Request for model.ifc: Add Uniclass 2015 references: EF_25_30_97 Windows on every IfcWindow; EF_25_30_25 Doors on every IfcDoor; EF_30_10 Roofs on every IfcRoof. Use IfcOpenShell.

First a look at what the model holds.

```python
import ifcopenshell

model = ifcopenshell.open("model.ifc")
print(model.schema)
print("classifications:", [c.Name for c in model.by_type("IfcClassification")])
for ifc_class in ("IfcDoor", "IfcRoof", "IfcStair", "IfcWall", "IfcWindow"):
    print(ifc_class, len(model.by_type(ifc_class)))
```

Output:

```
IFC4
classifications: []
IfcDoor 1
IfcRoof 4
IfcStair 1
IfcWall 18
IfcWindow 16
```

```python
import ifcopenshell
import ifcopenshell.api.classification

model = ifcopenshell.open("model.ifc")

system = ifcopenshell.api.classification.add_classification(model, classification="Uniclass 2015")

codes = {
    "IfcWindow": ("EF_25_30_97", "Windows"),
    "IfcDoor": ("EF_25_30_25", "Doors"),
    "IfcRoof": ("EF_30_10", "Roofs"),
}
for ifc_class, (code, name) in codes.items():
    products = model.by_type(ifc_class)
    ifcopenshell.api.classification.add_reference(
        model, products=products, classification=system, identification=code, name=name
    )
    print(code, len(products))

model.write("model_rev.ifc")
```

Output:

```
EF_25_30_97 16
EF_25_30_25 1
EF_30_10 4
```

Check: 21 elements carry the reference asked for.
